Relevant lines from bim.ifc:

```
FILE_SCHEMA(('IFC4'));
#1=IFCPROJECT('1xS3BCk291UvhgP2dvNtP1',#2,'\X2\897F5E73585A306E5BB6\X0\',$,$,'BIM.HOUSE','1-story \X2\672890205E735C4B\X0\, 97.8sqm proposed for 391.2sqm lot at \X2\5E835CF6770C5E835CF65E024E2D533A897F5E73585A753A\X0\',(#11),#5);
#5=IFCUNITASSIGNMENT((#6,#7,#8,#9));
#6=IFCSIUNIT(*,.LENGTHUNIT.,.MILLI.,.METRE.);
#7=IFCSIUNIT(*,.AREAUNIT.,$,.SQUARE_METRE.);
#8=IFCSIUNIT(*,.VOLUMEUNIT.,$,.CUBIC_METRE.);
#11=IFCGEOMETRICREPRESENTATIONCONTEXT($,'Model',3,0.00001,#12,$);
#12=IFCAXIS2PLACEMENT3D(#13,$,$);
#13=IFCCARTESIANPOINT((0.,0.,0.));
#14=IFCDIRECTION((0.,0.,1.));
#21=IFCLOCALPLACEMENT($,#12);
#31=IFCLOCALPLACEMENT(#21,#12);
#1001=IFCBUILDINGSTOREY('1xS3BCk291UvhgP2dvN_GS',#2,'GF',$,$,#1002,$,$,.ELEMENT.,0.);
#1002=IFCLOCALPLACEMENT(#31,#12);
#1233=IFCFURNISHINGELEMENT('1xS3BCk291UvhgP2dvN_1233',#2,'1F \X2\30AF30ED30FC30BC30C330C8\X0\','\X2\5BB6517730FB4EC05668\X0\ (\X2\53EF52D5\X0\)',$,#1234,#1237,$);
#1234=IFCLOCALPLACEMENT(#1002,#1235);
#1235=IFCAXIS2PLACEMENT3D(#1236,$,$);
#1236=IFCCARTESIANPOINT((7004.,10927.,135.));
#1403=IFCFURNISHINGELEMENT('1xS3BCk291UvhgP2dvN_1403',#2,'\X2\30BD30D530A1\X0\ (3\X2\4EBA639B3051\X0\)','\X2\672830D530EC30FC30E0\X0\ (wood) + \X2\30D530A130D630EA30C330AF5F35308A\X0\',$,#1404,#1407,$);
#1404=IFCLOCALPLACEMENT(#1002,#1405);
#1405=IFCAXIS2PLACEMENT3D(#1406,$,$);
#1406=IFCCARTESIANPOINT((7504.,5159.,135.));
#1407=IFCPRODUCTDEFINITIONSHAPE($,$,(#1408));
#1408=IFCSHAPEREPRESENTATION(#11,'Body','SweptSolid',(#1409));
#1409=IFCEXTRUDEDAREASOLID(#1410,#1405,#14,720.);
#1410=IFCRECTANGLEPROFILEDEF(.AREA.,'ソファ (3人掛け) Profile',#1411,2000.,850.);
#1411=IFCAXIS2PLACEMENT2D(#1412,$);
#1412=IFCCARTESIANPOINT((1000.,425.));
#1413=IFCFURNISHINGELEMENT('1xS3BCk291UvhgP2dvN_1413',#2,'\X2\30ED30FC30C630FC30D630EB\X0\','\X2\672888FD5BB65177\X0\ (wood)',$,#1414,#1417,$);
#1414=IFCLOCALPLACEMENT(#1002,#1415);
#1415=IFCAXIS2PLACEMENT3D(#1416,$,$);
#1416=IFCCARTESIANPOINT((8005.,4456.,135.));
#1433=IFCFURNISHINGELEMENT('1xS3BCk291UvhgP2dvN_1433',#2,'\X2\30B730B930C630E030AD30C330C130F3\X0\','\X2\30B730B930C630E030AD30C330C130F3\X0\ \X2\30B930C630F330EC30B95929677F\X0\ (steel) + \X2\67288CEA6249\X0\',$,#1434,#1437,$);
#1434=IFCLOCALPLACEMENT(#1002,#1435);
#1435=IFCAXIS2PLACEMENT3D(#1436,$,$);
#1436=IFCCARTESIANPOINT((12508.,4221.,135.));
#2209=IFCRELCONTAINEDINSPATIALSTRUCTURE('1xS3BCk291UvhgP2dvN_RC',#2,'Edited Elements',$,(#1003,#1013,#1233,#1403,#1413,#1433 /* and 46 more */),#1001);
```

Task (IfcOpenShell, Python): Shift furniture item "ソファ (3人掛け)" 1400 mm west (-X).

```python
import ifcopenshell
import ifcopenshell.api.geometry
import ifcopenshell.util.placement

model = ifcopenshell.open("bim.ifc")

item = model.by_guid("1xS3BCk291UvhgP2dvN_1403")
matrix = ifcopenshell.util.placement.get_local_placement(item.ObjectPlacement)
matrix[0, 3] -= 1400.0
ifcopenshell.api.geometry.edit_object_placement(model, product=item, matrix=matrix, is_si=False)

print(ifcopenshell.util.placement.get_local_placement(item.ObjectPlacement).round(3) + 0.0)

model.write("bim_v2.ifc")
```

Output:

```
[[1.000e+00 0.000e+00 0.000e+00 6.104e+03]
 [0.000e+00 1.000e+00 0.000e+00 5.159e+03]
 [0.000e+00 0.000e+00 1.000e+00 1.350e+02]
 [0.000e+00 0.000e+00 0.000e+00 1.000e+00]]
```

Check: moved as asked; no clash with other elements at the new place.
